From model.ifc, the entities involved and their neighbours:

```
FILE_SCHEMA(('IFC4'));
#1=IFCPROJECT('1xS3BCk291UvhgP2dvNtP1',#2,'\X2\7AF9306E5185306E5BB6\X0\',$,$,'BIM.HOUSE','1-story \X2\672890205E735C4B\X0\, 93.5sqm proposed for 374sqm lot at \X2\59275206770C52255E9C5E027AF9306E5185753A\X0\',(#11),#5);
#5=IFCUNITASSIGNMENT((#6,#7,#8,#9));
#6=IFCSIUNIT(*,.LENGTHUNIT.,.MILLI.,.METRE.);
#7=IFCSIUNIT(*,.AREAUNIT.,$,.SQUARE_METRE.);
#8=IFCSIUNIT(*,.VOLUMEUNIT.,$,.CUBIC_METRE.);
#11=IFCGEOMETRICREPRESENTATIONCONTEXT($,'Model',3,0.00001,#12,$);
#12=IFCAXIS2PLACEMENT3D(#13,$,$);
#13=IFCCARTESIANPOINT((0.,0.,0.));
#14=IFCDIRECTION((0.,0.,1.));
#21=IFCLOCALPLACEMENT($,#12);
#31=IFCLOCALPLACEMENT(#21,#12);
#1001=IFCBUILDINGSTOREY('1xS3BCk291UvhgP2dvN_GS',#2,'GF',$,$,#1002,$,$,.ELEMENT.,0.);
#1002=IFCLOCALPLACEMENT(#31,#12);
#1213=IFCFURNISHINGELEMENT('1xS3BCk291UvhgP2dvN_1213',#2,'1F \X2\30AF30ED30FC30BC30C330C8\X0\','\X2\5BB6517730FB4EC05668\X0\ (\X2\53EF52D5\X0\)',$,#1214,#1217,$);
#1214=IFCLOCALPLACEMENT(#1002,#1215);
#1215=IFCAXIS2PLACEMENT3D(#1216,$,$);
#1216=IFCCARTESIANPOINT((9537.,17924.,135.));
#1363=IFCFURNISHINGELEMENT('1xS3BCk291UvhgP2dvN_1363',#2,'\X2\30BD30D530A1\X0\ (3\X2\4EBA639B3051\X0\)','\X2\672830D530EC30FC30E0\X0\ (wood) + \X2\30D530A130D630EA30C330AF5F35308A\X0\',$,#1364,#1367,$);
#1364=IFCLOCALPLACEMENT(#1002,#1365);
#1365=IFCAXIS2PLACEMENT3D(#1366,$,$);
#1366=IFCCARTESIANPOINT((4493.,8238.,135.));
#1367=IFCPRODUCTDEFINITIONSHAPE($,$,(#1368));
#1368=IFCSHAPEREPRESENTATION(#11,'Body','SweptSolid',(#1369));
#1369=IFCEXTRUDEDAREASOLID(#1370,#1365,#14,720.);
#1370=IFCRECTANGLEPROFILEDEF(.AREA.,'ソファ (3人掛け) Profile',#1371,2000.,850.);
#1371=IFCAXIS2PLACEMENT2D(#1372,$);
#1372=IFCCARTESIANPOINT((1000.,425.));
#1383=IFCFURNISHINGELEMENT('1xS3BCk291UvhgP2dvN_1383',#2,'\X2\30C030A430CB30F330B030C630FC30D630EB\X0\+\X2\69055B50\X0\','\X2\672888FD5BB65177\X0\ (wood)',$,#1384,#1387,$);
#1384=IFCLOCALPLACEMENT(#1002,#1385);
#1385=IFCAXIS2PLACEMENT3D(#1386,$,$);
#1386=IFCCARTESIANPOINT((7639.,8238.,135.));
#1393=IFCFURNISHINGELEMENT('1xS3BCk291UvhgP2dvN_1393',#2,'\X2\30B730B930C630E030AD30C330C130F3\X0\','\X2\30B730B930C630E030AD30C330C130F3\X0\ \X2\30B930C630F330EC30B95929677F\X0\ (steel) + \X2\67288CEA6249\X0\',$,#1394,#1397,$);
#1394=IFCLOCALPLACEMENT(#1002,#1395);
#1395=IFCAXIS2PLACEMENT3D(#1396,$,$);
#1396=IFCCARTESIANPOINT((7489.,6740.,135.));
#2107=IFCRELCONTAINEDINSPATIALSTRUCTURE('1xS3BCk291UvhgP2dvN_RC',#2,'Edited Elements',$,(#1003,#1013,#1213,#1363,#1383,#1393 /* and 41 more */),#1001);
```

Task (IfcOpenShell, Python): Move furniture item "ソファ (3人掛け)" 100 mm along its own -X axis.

```python
import ifcopenshell
import ifcopenshell.api.geometry
import ifcopenshell.util.placement

model = ifcopenshell.open("model.ifc")

item = model.by_guid("1xS3BCk291UvhgP2dvN_1363")
matrix = ifcopenshell.util.placement.get_local_placement(item.ObjectPlacement)
matrix[:3, 3] -= matrix[:3, 0] * 100.0
ifcopenshell.api.geometry.edit_object_placement(model, product=item, matrix=matrix, is_si=False)

print(ifcopenshell.util.placement.get_local_placement(item.ObjectPlacement).round(3) + 0.0)

model.write("model_v2.ifc")
```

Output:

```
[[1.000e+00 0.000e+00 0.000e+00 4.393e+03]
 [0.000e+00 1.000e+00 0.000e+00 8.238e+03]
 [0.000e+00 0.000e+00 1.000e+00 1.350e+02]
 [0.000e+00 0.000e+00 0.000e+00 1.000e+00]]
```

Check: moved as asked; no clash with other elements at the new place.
